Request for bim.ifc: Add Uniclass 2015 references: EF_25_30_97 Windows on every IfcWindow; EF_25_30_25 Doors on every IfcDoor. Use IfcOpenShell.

First a look at what the model holds.

```python
import ifcopenshell

model = ifcopenshell.open("bim.ifc")
print(model.schema)
print("classifications:", [c.Name for c in model.by_type("IfcClassification")])
for ifc_class in ("IfcDoor", "IfcRoof", "IfcStair", "IfcWall", "IfcWindow"):
    print(ifc_class, len(model.by_type(ifc_class)))
```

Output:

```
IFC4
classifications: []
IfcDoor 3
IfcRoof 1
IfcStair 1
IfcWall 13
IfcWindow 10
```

```python
import ifcopenshell
import ifcopenshell.api.classification

model = ifcopenshell.open("bim.ifc")

system = ifcopenshell.api.classification.add_classification(model, classification="Uniclass 2015")

codes = {
    "IfcWindow": ("EF_25_30_97", "Windows"),
    "IfcDoor": ("EF_25_30_25", "Doors"),
}
for ifc_class, (code, name) in codes.items():
    products = model.by_type(ifc_class)
    ifcopenshell.api.classification.add_reference(
        model, products=products, classification=system, identification=code, name=name
    )
    print(code, len(products))

model.write("bim_v2.ifc")
```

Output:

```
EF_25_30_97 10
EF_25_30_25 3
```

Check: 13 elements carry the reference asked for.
